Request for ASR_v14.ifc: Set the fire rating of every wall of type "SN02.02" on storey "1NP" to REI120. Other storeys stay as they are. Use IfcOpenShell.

First a look at what the model holds.

```python
import ifcopenshell
import ifcopenshell.util.element

model = ifcopenshell.open("ASR_v14.ifc")
print(model.schema)
storey = next(s for s in model.by_type("IfcBuildingStorey") if s.Name == "1NP")
walls = [e for e in ifcopenshell.util.element.get_decomposition(storey) if e.is_a("IfcWall")]
seen = {}
for e in walls:
    element_type = ifcopenshell.util.element.get_type(e)
    key = (element_type.Name if element_type != e and element_type else None, ifcopenshell.util.element.get_pset(e, "Pset_WallCommon", "FireRating"))
    seen[key] = seen.get(key, 0) + 1
for (name, value), count in sorted(seen.items(), key=str):
    print(count, "x", name, "|", value)
```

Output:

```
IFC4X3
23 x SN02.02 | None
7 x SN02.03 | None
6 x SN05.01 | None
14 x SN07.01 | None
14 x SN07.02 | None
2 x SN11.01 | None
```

```python
import ifcopenshell
import ifcopenshell.api.pset
import ifcopenshell.util.element

model = ifcopenshell.open("ASR_v14.ifc")

storey = next(s for s in model.by_type("IfcBuildingStorey") if s.Name == "1NP")
walls = [e for e in ifcopenshell.util.element.get_decomposition(storey) if e.is_a("IfcWall")]

count = 0
for e in walls:
    element_type = ifcopenshell.util.element.get_type(e)
    if element_type in (None, e) or element_type.Name != "SN02.02":
        continue
    # add_pset returns the element's existing set when there is one.
    pset = ifcopenshell.api.pset.add_pset(model, product=e, name="Pset_WallCommon")
    ifcopenshell.api.pset.edit_pset(model, pset=pset, properties={"FireRating": "REI120"})
    count += 1

print(count, "walls updated")

model.write("ASR_v14_rev.ifc")
```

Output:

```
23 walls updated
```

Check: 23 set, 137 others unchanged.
